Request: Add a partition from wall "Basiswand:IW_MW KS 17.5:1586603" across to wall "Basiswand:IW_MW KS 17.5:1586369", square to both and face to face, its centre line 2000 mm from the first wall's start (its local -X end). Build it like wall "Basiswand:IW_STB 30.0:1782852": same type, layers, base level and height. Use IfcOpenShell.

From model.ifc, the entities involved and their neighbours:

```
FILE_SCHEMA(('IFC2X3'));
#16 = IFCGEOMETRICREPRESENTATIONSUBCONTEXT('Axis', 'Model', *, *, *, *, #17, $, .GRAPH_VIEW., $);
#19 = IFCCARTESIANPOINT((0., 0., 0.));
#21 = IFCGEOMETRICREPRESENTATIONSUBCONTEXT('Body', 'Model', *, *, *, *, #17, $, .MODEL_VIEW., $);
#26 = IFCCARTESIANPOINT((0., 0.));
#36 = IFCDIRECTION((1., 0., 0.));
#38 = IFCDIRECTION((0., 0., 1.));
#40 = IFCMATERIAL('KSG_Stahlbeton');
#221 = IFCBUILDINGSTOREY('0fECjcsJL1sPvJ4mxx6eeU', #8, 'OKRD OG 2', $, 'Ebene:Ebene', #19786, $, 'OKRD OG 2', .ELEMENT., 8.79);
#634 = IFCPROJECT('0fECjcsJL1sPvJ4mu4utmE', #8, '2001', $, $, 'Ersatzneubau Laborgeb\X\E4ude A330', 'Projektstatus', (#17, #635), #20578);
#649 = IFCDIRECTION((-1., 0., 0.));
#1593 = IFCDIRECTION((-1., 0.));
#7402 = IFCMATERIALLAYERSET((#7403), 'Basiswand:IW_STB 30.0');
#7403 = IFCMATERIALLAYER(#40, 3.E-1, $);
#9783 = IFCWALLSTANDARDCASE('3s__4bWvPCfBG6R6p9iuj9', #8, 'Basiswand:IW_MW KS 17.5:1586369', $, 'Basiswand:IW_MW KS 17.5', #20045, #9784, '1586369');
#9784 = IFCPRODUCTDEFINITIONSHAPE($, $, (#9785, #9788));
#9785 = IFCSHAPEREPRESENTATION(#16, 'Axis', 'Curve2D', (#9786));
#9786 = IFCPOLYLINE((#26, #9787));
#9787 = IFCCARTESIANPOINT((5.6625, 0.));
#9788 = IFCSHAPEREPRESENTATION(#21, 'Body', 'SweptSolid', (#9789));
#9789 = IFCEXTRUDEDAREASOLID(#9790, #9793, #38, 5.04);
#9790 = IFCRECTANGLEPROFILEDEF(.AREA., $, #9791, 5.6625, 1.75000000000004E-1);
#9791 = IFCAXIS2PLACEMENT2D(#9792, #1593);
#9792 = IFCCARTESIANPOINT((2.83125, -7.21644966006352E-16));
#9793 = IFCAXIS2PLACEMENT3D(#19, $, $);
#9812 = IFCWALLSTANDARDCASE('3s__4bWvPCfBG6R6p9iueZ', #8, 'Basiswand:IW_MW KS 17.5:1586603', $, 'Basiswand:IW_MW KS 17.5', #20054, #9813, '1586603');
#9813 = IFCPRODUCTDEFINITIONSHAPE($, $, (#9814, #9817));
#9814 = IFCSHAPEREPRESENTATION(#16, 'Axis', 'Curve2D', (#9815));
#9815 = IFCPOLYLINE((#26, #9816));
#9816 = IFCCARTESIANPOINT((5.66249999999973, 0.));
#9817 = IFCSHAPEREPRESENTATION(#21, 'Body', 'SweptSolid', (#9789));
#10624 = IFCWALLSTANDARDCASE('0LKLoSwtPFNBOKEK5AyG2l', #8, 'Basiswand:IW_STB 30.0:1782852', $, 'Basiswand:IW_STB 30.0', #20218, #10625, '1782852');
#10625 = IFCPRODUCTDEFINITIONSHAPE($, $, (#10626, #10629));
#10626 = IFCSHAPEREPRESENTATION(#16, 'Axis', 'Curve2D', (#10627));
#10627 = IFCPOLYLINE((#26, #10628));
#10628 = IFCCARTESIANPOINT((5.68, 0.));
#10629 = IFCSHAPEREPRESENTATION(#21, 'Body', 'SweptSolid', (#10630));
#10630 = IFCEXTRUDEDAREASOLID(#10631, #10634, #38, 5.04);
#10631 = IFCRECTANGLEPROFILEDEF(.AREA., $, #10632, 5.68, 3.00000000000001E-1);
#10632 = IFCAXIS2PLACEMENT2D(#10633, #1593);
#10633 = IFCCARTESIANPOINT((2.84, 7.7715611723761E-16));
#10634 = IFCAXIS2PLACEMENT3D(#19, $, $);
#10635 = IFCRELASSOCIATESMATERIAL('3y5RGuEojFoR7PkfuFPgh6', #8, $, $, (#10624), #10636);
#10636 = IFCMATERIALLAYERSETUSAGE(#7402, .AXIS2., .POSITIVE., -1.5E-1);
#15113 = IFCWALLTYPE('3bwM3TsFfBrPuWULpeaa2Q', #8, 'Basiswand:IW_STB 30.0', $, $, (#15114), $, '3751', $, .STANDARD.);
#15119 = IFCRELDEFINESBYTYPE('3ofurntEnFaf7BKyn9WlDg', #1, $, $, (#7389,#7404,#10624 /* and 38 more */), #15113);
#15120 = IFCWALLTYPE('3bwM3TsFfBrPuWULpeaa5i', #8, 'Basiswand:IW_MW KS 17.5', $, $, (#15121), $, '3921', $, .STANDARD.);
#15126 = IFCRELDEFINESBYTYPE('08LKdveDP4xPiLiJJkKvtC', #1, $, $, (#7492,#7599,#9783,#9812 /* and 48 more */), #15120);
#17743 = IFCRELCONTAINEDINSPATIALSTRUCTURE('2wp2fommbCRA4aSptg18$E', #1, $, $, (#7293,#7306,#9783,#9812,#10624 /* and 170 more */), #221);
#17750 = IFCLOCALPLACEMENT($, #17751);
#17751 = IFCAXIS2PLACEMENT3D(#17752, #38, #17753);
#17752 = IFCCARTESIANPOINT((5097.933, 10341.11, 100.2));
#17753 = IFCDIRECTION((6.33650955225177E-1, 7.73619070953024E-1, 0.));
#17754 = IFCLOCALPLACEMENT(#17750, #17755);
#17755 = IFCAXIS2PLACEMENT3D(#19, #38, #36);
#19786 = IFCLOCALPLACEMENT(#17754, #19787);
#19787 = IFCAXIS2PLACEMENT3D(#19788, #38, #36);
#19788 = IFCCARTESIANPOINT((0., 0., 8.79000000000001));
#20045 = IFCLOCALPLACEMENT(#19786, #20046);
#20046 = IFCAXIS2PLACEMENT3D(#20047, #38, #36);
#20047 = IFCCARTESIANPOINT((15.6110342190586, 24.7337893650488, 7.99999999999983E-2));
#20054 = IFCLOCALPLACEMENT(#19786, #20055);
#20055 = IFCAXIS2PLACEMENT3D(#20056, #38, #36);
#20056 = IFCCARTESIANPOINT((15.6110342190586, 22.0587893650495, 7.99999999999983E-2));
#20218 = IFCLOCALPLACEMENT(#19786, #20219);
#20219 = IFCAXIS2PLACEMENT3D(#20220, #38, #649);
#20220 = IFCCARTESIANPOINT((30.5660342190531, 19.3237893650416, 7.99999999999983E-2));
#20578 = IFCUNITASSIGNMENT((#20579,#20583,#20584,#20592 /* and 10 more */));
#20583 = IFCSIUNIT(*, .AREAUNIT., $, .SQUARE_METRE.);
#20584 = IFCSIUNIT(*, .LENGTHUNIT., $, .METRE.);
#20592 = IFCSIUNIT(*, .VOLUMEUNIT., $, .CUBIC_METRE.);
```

```python
import numpy as np
import ifcopenshell
import ifcopenshell.api.geometry
import ifcopenshell.api.material
import ifcopenshell.api.pset
import ifcopenshell.api.root
import ifcopenshell.api.spatial
import ifcopenshell.api.type
import ifcopenshell.geom
import ifcopenshell.util.element
import ifcopenshell.util.placement
import ifcopenshell.util.representation
import ifcopenshell.util.shape
import ifcopenshell.util.unit

model = ifcopenshell.open("model.ifc")
unit_scale = ifcopenshell.util.unit.calculate_unit_scale(model)
settings = ifcopenshell.geom.settings()
settings.set("use-world-coords", True)

start_wall = model.by_id(9812)
end_wall = model.by_guid("3s__4bWvPCfBG6R6p9iuj9")
like = model.by_guid("0LKLoSwtPFNBOKEK5AyG2l")
matrix = ifcopenshell.util.placement.get_local_placement(start_wall.ObjectPlacement)
matrix[:3, 3] *= unit_scale


def extent(element):
    """Bounding box in the first wall's axes, in metres."""
    shape = ifcopenshell.geom.create_shape(settings, element)
    points = (ifcopenshell.util.shape.get_vertices(shape.geometry) - matrix[:3, 3]) @ matrix[:3, :3]
    return points.min(axis=0), points.max(axis=0)


y_start = extent(start_wall)[1][1]
y_end = extent(end_wall)[0][1]
like_min, like_max = extent(like)
length, height = float(abs(y_end - y_start)), float(like_max[2] - like_min[2])
layer_set = ifcopenshell.util.element.get_material(like, should_skip_usage=True)
thickness = sum(layer.LayerThickness for layer in layer_set.MaterialLayers) * unit_scale

wall = ifcopenshell.api.root.create_entity(model, ifc_class="IfcWallStandardCase", name="New partition")
storey = ifcopenshell.util.element.get_container(like)
ifcopenshell.api.spatial.assign_container(model, products=[wall], relating_structure=storey)
ifcopenshell.api.type.assign_type(
    model, related_objects=[wall], relating_type=ifcopenshell.util.element.get_type(like), should_map_representations=False
)
rel = ifcopenshell.api.material.assign_material(
    model, products=[wall], type="IfcMaterialLayerSetUsage", material=layer_set
)
rel.RelatingMaterial.OffsetFromReferenceLine = -thickness / 2 / unit_scale
pset = ifcopenshell.api.pset.add_pset(model, product=wall, name="Pset_WallCommon")
ifcopenshell.api.pset.edit_pset(model, pset=pset, properties={"IsExternal": False, "LoadBearing": False})

# The axis runs down the middle of the wall.
axis = ifcopenshell.api.geometry.add_axis_representation(
    model, context=ifcopenshell.util.representation.get_context(model, "Model", "Axis"), axis=[(0.0, 0.0), (length, 0.0)]
)
body = ifcopenshell.api.geometry.add_wall_representation(
    model,
    context=ifcopenshell.util.representation.get_context(model, "Model", "Body", "MODEL_VIEW"),
    length=length,
    height=height,
    thickness=thickness,
    offset=-thickness / 2,
)
for representation in (axis, body):
    ifcopenshell.api.geometry.assign_representation(model, product=wall, representation=representation)

placement = matrix @ ifcopenshell.util.placement.rotation(90, "Z")
placement[:, 3] = matrix @ np.array([extent(start_wall)[0][0] + 2, y_start, like_min[2], 1.0])
ifcopenshell.api.geometry.edit_object_placement(model, product=wall, matrix=placement)

print(f"partition {length:.3f} m long, {height:.3f} m high, {thickness:.3f} m thick")

model.write("model_edited.ifc")
```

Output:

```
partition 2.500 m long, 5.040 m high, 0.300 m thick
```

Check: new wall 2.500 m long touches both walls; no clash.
